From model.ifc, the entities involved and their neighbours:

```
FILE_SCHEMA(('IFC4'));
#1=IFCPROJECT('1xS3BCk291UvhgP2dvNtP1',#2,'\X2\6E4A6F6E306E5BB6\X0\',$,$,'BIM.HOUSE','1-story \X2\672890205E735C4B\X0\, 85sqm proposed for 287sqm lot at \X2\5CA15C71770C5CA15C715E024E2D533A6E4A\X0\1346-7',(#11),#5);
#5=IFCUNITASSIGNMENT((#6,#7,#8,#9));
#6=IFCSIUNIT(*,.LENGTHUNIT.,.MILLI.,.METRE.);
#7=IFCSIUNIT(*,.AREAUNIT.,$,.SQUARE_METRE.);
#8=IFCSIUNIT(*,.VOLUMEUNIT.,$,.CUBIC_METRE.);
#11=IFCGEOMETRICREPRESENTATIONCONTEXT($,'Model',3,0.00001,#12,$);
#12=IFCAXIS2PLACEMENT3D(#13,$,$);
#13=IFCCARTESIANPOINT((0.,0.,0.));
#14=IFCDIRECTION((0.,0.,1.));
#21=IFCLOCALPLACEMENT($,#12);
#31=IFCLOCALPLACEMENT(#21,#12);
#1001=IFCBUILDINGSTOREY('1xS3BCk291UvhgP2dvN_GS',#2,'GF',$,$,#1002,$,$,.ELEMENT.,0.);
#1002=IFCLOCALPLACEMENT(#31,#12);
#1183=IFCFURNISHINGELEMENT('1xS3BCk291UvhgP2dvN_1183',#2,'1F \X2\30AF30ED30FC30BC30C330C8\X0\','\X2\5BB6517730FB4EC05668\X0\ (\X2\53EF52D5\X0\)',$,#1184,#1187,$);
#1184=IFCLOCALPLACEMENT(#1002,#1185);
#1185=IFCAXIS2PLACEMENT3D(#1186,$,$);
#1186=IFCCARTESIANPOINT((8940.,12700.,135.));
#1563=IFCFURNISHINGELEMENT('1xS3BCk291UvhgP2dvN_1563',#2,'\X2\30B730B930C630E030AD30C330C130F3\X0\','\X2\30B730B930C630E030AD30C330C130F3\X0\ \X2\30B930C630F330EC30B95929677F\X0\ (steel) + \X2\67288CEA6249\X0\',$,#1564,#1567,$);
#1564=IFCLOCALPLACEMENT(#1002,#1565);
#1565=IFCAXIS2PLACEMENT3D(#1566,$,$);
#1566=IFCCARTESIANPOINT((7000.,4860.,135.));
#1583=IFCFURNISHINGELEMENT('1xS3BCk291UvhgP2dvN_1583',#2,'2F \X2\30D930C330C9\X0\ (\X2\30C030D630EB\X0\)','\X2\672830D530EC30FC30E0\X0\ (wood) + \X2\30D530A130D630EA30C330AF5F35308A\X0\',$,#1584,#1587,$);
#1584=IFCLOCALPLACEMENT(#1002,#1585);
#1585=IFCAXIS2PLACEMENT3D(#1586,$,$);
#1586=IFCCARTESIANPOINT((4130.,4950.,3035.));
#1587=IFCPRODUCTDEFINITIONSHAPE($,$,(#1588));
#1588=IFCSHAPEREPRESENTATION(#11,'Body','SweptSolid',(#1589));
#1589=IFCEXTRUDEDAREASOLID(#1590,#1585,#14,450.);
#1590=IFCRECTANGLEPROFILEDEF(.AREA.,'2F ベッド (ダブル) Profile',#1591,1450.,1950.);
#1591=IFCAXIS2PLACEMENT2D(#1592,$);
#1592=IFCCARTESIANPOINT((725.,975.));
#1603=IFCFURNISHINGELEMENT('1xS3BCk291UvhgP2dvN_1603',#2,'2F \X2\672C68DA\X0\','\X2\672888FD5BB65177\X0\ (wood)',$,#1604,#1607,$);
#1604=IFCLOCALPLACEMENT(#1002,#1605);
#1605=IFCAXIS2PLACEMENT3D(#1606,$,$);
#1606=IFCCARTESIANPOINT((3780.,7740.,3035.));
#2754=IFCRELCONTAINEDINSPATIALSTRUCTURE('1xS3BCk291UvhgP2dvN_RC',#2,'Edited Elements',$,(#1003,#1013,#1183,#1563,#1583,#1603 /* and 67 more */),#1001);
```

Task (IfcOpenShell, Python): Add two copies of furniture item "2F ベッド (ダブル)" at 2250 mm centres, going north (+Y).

```python
import numpy as np
import ifcopenshell
import ifcopenshell.api.geometry
import ifcopenshell.api.root
import ifcopenshell.util.element
import ifcopenshell.util.placement
import ifcopenshell.util.unit

model = ifcopenshell.open("model.ifc")
unit_scale = ifcopenshell.util.unit.calculate_unit_scale(model)


def reuse_history(source, copy):
    """copy_class also copies each property set's owner history, people and application; keep the originals."""
    for rel in copy.IsDefinedBy:
        if rel.is_a("IfcRelDefinesByProperties") and (history := rel.RelatingPropertyDefinition.OwnerHistory):
            rel.RelatingPropertyDefinition.OwnerHistory = source.OwnerHistory
            ifcopenshell.util.element.remove_deep2(model, history)


source = model.by_guid("1xS3BCk291UvhgP2dvN_1583")
base = ifcopenshell.util.placement.get_local_placement(source.ObjectPlacement)
step = np.array([0.0, 1.0, 0.0]) * 2.25 / unit_scale

for i in range(1, 3):
    copy = ifcopenshell.api.root.copy_class(model, product=source)
    copy.Representation = ifcopenshell.util.element.copy_deep(
        model, source.Representation, exclude=["IfcGeometricRepresentationContext", "IfcRepresentationMap"]
    )
    reuse_history(source, copy)
    matrix = base.copy()
    matrix[:3, 3] += i * step
    print("added at", matrix[:3, 3].round(3) + 0.0)
    ifcopenshell.api.geometry.edit_object_placement(model, product=copy, matrix=matrix, is_si=False)

model.write("model_rev.ifc")
```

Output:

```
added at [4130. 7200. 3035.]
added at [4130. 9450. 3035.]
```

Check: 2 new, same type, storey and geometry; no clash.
